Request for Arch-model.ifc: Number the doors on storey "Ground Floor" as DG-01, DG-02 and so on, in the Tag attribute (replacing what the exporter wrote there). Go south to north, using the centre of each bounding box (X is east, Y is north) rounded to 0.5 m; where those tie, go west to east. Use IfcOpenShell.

First a look at what the model holds.

```python
import ifcopenshell
import ifcopenshell.util.element
import ifcopenshell.util.placement

model = ifcopenshell.open("Arch-model.ifc")
print(model.schema)
storey = next(s for s in model.by_type("IfcBuildingStorey") if s.Name == "Ground Floor")
doors = [e for e in ifcopenshell.util.element.get_decomposition(storey) if e.is_a("IfcDoor")]
for e in sorted(doors, key=lambda e: e.id()):
    origin = ifcopenshell.util.placement.get_local_placement(e.ObjectPlacement)[:3, 3]
    print(e.id(), e.Tag, e.Name, origin.round(2) + 0.0, sep=" | ")
```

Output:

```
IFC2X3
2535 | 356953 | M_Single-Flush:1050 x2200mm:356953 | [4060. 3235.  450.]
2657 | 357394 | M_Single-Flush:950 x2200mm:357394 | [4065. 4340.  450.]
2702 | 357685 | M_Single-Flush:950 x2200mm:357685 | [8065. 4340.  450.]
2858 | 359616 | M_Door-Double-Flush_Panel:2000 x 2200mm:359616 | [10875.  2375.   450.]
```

```python
import ifcopenshell
import ifcopenshell.geom
import ifcopenshell.util.element
import ifcopenshell.util.shape

model = ifcopenshell.open("Arch-model.ifc")
settings = ifcopenshell.geom.settings()
settings.set("use-world-coords", True)


def centre(element):
    shape = ifcopenshell.geom.create_shape(settings, element)
    return ifcopenshell.util.shape.get_bbox_centroid(shape.geometry)


storey = next(s for s in model.by_type("IfcBuildingStorey") if s.Name == "Ground Floor")
doors = [e for e in ifcopenshell.util.element.get_decomposition(storey) if e.is_a("IfcDoor")]

# Insertion points can sit at a corner or the storey origin, so sort by the geometry (in metres).
centres = {e: centre(e) for e in doors}
doors.sort(key=lambda e: (round(centres[e][1] / 0.5), centres[e][0]))

for i, e in enumerate(doors, start=1):
    number = f"DG-{i:02d}"
    e.Tag = number
    print(e.id(), number)

model.write("Arch-model_edited.ifc")
```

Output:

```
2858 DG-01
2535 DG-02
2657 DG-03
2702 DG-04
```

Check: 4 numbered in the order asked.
